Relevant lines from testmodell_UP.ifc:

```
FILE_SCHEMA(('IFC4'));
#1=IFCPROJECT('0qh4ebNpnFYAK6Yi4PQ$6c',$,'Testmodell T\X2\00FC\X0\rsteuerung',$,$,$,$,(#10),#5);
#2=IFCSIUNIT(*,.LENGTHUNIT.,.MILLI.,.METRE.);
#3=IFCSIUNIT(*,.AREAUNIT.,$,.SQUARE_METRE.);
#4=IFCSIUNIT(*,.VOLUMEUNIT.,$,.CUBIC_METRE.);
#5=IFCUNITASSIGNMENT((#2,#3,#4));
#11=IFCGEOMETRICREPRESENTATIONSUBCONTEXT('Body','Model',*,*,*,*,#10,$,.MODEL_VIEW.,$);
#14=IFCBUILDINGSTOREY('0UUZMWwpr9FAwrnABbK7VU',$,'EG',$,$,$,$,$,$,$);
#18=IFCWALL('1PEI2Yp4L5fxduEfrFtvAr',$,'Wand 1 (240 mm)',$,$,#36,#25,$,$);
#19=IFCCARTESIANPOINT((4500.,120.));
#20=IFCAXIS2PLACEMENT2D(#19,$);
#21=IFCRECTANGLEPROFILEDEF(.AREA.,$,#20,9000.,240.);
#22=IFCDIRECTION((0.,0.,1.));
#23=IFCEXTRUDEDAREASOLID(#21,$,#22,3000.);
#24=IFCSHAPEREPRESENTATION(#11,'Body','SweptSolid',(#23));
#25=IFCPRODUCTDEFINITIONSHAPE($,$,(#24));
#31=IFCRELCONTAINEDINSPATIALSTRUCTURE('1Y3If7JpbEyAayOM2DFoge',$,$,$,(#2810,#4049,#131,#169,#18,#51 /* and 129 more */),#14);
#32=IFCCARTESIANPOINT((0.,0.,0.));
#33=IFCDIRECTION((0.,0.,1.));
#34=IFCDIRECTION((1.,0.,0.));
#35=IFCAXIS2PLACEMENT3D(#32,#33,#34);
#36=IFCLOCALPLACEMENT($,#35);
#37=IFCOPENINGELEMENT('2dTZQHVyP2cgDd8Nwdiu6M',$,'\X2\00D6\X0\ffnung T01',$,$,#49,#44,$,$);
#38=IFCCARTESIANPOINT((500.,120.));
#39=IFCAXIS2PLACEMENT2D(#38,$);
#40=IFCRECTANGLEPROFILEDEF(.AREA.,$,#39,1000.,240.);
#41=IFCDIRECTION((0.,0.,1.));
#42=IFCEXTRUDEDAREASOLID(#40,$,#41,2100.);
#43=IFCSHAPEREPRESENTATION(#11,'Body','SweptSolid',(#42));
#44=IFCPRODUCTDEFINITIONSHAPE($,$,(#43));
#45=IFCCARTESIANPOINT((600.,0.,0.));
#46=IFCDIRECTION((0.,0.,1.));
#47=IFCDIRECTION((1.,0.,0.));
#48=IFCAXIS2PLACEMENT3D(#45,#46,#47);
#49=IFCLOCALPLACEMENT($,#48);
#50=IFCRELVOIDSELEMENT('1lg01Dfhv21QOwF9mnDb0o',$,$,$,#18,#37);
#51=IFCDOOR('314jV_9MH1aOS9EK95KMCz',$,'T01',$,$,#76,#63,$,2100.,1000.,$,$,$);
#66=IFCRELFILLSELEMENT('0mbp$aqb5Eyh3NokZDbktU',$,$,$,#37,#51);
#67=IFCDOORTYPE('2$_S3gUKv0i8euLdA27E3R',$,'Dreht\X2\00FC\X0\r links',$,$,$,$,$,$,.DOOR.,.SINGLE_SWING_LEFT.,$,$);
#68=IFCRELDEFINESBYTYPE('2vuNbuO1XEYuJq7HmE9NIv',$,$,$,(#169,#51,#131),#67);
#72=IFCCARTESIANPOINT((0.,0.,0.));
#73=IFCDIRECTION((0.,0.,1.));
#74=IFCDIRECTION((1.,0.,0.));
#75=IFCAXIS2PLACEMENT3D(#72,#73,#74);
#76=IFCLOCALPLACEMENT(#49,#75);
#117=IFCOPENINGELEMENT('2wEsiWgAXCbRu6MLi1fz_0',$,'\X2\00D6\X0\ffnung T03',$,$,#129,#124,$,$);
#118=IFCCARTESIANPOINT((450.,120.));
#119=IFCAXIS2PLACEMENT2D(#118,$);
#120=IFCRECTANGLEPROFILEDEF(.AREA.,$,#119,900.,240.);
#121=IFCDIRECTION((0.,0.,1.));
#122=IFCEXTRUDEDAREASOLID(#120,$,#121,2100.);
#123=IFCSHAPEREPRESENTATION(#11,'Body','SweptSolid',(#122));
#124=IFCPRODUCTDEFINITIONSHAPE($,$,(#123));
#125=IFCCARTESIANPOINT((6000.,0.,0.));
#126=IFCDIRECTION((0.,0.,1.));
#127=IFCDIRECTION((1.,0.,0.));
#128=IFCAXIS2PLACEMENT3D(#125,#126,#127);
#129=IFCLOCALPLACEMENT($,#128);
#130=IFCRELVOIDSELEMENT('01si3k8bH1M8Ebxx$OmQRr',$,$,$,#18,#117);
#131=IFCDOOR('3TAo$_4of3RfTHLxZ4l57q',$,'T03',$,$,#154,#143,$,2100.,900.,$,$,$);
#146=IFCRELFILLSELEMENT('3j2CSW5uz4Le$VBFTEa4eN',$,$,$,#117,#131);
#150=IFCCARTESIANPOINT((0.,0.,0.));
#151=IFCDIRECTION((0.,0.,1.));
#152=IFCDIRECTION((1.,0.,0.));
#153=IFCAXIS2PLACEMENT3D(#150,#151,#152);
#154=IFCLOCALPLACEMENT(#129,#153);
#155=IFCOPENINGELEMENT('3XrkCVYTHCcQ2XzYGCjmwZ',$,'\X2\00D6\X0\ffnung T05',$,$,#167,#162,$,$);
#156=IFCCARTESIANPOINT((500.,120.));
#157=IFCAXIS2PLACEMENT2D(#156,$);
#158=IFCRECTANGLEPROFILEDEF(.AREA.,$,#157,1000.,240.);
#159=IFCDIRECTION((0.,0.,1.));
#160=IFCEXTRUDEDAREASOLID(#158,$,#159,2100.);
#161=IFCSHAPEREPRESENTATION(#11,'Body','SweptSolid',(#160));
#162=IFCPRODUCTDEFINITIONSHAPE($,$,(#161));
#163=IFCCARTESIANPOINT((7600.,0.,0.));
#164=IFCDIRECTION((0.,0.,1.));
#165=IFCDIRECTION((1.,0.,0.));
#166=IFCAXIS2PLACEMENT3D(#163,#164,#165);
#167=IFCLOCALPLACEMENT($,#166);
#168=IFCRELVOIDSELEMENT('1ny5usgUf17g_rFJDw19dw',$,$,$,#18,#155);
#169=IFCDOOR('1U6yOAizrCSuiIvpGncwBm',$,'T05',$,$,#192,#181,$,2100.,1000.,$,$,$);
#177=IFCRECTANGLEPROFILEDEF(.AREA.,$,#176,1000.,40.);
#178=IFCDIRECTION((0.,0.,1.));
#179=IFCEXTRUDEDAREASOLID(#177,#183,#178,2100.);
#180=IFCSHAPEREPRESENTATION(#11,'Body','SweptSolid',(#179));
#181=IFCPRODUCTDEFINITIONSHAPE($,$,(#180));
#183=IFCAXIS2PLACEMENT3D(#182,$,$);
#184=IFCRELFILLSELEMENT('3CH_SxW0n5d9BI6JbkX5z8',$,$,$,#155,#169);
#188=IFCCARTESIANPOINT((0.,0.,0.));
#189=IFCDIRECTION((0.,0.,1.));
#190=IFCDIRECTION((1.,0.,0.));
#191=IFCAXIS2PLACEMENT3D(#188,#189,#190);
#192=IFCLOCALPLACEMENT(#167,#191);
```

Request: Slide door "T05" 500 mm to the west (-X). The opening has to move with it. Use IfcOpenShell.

```python
import ifcopenshell
import ifcopenshell.api.geometry
import ifcopenshell.util.placement
import ifcopenshell.util.unit

model = ifcopenshell.open("testmodell_UP.ifc")
unit_scale = ifcopenshell.util.unit.calculate_unit_scale(model)

door = model.by_guid("1U6yOAizrCSuiIvpGncwBm")
opening = door.FillsVoids[0].RelatingOpeningElement
wall = opening.VoidsElements[0].RelatingBuildingElement

wall_matrix = ifcopenshell.util.placement.get_local_placement(wall.ObjectPlacement)
shift = wall_matrix[:3, 0] * -0.5 / unit_scale
before = ifcopenshell.util.placement.get_local_placement(door.ObjectPlacement)[:3, 3].copy()

# The door is placed relative to its opening, so it follows when the opening moves.
matrix = ifcopenshell.util.placement.get_local_placement(opening.ObjectPlacement)
matrix[:3, 3] += shift
ifcopenshell.api.geometry.edit_object_placement(
    model, product=opening, matrix=matrix, is_si=False, should_transform_children=True
)

after = ifcopenshell.util.placement.get_local_placement(door.ObjectPlacement)[:3, 3]
print("door moved by", (after - before).round(3) + 0.0)

model.write("testmodell_UP_edited.ifc")
```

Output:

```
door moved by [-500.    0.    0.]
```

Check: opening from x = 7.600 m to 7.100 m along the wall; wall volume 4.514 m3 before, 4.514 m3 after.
